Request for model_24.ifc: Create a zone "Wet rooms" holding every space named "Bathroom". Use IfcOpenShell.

First a look at what the model holds.

```python
import ifcopenshell

model = ifcopenshell.open("model_24.ifc")
print(model.schema)
seen = {}
for space in model.by_type("IfcSpace"):
    seen[space.LongName] = seen.get(space.LongName, 0) + 1
for name, count in sorted(seen.items(), key=str):
    print(count, "x", name)
print("zones:", [z.Name for z in model.by_type("IfcZone")][:20])
```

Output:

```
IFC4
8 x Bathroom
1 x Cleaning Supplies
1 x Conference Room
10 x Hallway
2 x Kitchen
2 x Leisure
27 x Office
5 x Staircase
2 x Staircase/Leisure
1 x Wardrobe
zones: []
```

```python
import ifcopenshell
import ifcopenshell.api.group
import ifcopenshell.api.root

model = ifcopenshell.open("model_24.ifc")

names = {"Bathroom"}
spaces = [s for s in model.by_type("IfcSpace") if s.LongName in names]

zone = ifcopenshell.api.root.create_entity(model, ifc_class="IfcZone", name="Wet rooms")
ifcopenshell.api.group.assign_group(model, products=spaces, group=zone)
print(len(spaces), "spaces in", zone.Name)

model.write("model_24_updated.ifc")
```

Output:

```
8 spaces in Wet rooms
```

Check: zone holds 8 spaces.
